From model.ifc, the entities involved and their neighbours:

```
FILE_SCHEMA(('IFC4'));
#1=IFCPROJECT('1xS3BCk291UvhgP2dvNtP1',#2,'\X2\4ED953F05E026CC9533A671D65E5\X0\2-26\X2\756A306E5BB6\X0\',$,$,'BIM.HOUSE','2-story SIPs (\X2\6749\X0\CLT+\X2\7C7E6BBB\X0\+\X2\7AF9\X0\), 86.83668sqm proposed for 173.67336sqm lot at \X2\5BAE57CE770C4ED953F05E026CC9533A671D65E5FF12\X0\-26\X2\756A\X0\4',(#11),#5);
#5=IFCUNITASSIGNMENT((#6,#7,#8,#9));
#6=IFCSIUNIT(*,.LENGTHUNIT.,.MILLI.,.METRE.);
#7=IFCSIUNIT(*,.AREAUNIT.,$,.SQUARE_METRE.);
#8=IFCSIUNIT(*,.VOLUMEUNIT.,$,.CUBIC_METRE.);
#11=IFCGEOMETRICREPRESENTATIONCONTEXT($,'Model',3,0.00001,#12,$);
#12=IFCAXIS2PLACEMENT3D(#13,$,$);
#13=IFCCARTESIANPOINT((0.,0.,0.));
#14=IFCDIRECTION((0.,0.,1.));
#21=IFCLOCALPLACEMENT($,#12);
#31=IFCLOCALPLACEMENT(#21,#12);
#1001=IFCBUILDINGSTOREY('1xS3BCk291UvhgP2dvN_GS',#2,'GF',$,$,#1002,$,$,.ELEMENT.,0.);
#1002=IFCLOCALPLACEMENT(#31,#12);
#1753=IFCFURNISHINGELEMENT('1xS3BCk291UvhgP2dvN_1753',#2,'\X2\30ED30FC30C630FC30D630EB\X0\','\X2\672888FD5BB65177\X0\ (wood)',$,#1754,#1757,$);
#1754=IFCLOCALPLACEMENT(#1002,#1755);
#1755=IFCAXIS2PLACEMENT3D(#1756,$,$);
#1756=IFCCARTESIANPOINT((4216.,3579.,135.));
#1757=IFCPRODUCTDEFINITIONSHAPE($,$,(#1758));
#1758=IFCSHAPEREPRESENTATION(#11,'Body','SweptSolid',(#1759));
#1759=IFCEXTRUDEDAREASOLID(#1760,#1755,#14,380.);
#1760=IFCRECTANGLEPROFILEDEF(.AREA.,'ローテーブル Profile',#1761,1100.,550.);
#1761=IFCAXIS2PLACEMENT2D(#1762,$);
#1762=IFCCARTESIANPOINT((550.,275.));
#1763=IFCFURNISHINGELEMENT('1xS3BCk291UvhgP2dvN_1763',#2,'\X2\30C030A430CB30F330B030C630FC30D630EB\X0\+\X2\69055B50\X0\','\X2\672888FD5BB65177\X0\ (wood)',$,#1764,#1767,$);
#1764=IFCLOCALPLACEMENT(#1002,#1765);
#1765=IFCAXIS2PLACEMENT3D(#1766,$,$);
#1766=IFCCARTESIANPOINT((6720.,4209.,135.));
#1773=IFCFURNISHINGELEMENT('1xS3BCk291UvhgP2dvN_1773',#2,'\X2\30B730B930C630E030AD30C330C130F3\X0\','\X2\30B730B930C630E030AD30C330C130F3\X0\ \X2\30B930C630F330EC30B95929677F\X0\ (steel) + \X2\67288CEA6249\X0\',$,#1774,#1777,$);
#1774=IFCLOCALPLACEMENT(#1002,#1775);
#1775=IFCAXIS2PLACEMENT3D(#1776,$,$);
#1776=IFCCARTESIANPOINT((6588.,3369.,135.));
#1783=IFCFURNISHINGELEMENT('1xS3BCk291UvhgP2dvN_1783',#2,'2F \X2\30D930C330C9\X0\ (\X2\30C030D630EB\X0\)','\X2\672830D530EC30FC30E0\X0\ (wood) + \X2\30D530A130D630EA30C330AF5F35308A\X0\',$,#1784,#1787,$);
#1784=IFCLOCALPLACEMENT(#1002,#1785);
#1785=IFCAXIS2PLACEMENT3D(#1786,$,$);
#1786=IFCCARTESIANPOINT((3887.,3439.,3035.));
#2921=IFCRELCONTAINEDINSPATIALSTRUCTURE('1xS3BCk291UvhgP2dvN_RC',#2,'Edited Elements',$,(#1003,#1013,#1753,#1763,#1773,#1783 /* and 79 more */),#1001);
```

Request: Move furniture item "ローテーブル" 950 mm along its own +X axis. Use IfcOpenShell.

```python
import ifcopenshell
import ifcopenshell.api.geometry
import ifcopenshell.util.placement
import ifcopenshell.util.unit

model = ifcopenshell.open("model.ifc")
unit_scale = ifcopenshell.util.unit.calculate_unit_scale(model)

item = model.by_guid("1xS3BCk291UvhgP2dvN_1753")
matrix = ifcopenshell.util.placement.get_local_placement(item.ObjectPlacement)
matrix[:3, 3] += matrix[:3, 0] * 0.95 / unit_scale
ifcopenshell.api.geometry.edit_object_placement(model, product=item, matrix=matrix, is_si=False)

print(ifcopenshell.util.placement.get_local_placement(item.ObjectPlacement).round(3) + 0.0)

model.write("model-out.ifc")
```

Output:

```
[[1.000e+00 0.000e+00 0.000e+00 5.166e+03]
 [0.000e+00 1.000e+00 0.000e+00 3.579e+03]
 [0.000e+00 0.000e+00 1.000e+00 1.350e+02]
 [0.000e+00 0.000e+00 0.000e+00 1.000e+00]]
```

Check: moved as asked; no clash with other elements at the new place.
